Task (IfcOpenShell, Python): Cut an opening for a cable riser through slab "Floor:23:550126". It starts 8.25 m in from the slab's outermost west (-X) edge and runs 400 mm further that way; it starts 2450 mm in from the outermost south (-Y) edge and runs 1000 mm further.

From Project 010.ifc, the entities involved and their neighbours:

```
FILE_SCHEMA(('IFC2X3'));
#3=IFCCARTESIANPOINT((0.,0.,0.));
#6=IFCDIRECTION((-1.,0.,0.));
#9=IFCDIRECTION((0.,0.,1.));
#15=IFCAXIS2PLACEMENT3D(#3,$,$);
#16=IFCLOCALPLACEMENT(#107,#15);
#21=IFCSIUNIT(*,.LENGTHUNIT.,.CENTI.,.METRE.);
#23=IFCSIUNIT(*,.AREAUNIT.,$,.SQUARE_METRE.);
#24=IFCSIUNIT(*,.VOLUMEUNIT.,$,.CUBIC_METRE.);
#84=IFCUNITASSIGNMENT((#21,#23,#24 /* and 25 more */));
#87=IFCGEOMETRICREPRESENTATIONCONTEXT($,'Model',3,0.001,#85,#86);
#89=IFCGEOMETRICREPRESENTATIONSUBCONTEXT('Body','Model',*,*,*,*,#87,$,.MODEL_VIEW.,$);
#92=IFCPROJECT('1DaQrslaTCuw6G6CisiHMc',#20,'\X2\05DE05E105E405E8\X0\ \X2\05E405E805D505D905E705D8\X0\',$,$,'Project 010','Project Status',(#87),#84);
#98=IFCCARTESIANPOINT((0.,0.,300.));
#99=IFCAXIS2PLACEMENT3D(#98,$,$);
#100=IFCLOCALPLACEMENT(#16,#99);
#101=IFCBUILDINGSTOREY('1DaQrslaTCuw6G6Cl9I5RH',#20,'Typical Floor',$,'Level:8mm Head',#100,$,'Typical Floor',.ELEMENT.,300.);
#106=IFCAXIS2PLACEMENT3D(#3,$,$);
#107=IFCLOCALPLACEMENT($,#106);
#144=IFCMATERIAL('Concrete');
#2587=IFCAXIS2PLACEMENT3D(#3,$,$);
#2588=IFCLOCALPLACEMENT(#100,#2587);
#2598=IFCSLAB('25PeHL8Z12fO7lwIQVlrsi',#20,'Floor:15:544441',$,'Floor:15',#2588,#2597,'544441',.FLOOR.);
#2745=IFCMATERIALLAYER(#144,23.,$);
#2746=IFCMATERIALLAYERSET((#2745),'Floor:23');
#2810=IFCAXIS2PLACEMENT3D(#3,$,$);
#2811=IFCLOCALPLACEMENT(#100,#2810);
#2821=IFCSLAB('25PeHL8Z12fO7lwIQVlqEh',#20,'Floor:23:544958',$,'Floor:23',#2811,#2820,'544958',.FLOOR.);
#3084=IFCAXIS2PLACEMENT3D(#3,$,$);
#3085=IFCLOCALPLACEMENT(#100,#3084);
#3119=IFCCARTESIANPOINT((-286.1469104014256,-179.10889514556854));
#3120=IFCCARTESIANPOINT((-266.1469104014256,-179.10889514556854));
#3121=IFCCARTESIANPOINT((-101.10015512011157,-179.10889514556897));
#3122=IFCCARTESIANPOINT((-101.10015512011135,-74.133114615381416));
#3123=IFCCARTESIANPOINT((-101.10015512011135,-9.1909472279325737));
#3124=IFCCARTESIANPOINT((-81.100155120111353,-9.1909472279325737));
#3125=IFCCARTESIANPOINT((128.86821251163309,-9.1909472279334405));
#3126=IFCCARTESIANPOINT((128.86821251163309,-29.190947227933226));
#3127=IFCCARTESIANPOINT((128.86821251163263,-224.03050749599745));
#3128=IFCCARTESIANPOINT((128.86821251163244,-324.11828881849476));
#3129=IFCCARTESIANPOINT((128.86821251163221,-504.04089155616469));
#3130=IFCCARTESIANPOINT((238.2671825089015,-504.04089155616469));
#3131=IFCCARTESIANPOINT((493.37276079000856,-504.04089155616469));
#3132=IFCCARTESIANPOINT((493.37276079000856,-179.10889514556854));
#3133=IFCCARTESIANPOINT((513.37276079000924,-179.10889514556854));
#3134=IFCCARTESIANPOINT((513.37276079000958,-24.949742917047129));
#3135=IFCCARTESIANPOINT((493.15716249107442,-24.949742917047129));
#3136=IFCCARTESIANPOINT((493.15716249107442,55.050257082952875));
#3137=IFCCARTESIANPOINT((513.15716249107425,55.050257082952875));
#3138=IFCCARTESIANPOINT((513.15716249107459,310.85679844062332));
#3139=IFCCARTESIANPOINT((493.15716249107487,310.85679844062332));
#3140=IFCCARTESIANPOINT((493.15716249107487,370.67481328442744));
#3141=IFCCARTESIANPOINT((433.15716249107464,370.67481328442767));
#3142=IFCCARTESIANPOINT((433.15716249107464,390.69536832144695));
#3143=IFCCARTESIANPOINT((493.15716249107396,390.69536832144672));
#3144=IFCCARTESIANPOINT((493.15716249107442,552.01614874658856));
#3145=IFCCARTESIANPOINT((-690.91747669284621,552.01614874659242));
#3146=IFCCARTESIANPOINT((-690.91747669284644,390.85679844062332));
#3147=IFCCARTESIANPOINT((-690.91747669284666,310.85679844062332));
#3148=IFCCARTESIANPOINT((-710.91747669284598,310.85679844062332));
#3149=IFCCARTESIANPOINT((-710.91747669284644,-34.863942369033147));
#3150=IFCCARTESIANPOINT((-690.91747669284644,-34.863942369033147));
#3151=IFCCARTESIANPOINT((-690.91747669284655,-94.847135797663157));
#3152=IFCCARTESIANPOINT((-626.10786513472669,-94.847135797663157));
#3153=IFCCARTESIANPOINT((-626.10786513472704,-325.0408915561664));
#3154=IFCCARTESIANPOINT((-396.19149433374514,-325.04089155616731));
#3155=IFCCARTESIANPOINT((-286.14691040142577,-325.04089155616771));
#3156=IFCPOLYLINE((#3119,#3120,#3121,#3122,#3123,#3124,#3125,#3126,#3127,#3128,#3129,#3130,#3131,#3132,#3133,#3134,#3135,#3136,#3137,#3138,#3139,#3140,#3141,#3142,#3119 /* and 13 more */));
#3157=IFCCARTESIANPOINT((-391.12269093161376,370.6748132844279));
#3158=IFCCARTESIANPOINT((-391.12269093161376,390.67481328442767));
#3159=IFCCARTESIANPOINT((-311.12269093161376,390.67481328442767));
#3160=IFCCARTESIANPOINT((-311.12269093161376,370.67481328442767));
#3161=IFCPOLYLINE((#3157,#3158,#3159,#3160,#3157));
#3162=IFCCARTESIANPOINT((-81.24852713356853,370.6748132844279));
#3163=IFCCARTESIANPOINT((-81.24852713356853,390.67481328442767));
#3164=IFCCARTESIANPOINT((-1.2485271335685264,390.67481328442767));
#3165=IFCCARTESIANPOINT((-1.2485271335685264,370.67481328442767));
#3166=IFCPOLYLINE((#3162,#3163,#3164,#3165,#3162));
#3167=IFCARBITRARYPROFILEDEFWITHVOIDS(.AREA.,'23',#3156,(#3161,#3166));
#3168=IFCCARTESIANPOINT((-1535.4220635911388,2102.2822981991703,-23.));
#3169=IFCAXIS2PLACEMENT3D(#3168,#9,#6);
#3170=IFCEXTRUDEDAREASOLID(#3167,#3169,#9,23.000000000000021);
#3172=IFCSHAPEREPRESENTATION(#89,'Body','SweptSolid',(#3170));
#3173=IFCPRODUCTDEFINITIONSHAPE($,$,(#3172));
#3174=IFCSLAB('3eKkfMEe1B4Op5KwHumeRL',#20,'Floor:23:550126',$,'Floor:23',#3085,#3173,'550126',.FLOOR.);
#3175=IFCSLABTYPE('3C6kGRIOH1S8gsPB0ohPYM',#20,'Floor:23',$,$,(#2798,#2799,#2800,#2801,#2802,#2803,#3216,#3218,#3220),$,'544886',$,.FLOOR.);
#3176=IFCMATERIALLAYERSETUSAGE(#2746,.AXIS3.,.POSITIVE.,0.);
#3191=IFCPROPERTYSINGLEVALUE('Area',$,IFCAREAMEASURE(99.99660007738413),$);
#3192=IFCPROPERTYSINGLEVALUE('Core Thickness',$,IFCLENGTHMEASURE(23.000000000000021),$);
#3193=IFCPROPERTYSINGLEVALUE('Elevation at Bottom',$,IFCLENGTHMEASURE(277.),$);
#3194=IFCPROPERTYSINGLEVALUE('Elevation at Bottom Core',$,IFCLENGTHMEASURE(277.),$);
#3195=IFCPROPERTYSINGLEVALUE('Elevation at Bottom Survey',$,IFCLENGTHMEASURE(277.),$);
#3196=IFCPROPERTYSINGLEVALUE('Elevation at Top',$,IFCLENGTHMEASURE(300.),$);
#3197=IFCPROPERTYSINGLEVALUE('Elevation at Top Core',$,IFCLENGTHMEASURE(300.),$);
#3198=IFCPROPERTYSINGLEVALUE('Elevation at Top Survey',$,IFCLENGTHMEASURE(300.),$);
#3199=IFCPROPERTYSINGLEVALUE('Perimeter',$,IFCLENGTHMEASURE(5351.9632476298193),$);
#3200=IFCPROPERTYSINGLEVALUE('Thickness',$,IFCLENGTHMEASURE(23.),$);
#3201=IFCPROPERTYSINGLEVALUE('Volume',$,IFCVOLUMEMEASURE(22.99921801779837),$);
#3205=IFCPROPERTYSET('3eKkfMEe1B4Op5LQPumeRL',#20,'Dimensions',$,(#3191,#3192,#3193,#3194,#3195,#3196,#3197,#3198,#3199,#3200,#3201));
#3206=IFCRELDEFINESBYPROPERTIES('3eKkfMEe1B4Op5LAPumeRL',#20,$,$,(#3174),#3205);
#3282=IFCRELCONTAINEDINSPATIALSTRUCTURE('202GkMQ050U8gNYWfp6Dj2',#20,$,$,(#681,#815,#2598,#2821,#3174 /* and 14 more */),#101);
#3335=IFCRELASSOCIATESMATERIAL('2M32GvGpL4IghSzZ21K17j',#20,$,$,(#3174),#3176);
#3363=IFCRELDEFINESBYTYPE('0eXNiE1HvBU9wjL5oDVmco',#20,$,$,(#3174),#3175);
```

```python
import numpy as np
import ifcopenshell
import ifcopenshell.api.feature
import ifcopenshell.api.geometry
import ifcopenshell.api.pset
import ifcopenshell.api.root
import ifcopenshell.geom
import ifcopenshell.util.element
import ifcopenshell.util.placement
import ifcopenshell.util.representation
import ifcopenshell.util.shape
import ifcopenshell.util.unit

model = ifcopenshell.open("Project 010.ifc")
unit_scale = ifcopenshell.util.unit.calculate_unit_scale(model)
area_scale = ifcopenshell.util.unit.calculate_unit_scale(model, "AREAUNIT")
volume_scale = ifcopenshell.util.unit.calculate_unit_scale(model, "VOLUMEUNIT")
settings = ifcopenshell.geom.settings()


def volume(element):
    """Net volume in cubic metres, openings subtracted."""
    shape = ifcopenshell.geom.create_shape(settings, element)
    return ifcopenshell.util.shape.get_volume(shape.geometry)


slab = model.by_guid("3eKkfMEe1B4Op5KwHumeRL")
before = volume(slab)

# Extent in the slab's own axes, in metres. The edges named are its -X and -Y sides.
slab_shape = ifcopenshell.geom.create_shape(settings, slab)
vertices = ifcopenshell.util.shape.get_vertices(slab_shape.geometry)
x_min, y_min, bottom = vertices.min(axis=0)
top = vertices[:, 2].max()

opening = ifcopenshell.api.root.create_entity(model, ifc_class="IfcOpeningElement", name="Cable riser opening")
context = ifcopenshell.util.representation.get_context(model, "Model", "Body", "MODEL_VIEW")
width, depth = 0.4, 1
outline = [(0.0, 0.0), (width, 0.0), (width, depth), (0.0, depth), (0.0, 0.0)]
# Overshoot both faces by 50 mm so the cut is clean.
shape = ifcopenshell.api.geometry.add_slab_representation(
    model, context=context, depth=top - bottom + 0.1, polyline=outline
)
ifcopenshell.api.geometry.assign_representation(model, product=opening, representation=shape)

matrix = ifcopenshell.util.placement.get_local_placement(slab.ObjectPlacement)
matrix[:, 3] = matrix @ np.append(np.array([x_min + 8.25, y_min + 2.45, bottom - 0.05]) / unit_scale, 1.0)
ifcopenshell.api.geometry.edit_object_placement(model, product=opening, matrix=matrix, is_si=False)
ifcopenshell.api.feature.add_feature(model, feature=opening, element=slab)

after = volume(slab)

# Update the slab's stored quantities.
pset = model.by_id(ifcopenshell.util.element.get_pset(slab, "Dimensions", should_inherit=False)["id"])
ifcopenshell.api.pset.edit_pset(model, pset=pset, properties={
    "Area": model.create_entity("IfcAreaMeasure", after / (top - bottom) / area_scale),
    "Volume": model.create_entity("IfcVolumeMeasure", after / volume_scale),
})

print(f"slab volume {before:.3f} -> {after:.3f} m3")

model.write("Project 010_edited.ifc")
```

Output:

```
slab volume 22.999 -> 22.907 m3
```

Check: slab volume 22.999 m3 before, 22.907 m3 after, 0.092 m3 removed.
